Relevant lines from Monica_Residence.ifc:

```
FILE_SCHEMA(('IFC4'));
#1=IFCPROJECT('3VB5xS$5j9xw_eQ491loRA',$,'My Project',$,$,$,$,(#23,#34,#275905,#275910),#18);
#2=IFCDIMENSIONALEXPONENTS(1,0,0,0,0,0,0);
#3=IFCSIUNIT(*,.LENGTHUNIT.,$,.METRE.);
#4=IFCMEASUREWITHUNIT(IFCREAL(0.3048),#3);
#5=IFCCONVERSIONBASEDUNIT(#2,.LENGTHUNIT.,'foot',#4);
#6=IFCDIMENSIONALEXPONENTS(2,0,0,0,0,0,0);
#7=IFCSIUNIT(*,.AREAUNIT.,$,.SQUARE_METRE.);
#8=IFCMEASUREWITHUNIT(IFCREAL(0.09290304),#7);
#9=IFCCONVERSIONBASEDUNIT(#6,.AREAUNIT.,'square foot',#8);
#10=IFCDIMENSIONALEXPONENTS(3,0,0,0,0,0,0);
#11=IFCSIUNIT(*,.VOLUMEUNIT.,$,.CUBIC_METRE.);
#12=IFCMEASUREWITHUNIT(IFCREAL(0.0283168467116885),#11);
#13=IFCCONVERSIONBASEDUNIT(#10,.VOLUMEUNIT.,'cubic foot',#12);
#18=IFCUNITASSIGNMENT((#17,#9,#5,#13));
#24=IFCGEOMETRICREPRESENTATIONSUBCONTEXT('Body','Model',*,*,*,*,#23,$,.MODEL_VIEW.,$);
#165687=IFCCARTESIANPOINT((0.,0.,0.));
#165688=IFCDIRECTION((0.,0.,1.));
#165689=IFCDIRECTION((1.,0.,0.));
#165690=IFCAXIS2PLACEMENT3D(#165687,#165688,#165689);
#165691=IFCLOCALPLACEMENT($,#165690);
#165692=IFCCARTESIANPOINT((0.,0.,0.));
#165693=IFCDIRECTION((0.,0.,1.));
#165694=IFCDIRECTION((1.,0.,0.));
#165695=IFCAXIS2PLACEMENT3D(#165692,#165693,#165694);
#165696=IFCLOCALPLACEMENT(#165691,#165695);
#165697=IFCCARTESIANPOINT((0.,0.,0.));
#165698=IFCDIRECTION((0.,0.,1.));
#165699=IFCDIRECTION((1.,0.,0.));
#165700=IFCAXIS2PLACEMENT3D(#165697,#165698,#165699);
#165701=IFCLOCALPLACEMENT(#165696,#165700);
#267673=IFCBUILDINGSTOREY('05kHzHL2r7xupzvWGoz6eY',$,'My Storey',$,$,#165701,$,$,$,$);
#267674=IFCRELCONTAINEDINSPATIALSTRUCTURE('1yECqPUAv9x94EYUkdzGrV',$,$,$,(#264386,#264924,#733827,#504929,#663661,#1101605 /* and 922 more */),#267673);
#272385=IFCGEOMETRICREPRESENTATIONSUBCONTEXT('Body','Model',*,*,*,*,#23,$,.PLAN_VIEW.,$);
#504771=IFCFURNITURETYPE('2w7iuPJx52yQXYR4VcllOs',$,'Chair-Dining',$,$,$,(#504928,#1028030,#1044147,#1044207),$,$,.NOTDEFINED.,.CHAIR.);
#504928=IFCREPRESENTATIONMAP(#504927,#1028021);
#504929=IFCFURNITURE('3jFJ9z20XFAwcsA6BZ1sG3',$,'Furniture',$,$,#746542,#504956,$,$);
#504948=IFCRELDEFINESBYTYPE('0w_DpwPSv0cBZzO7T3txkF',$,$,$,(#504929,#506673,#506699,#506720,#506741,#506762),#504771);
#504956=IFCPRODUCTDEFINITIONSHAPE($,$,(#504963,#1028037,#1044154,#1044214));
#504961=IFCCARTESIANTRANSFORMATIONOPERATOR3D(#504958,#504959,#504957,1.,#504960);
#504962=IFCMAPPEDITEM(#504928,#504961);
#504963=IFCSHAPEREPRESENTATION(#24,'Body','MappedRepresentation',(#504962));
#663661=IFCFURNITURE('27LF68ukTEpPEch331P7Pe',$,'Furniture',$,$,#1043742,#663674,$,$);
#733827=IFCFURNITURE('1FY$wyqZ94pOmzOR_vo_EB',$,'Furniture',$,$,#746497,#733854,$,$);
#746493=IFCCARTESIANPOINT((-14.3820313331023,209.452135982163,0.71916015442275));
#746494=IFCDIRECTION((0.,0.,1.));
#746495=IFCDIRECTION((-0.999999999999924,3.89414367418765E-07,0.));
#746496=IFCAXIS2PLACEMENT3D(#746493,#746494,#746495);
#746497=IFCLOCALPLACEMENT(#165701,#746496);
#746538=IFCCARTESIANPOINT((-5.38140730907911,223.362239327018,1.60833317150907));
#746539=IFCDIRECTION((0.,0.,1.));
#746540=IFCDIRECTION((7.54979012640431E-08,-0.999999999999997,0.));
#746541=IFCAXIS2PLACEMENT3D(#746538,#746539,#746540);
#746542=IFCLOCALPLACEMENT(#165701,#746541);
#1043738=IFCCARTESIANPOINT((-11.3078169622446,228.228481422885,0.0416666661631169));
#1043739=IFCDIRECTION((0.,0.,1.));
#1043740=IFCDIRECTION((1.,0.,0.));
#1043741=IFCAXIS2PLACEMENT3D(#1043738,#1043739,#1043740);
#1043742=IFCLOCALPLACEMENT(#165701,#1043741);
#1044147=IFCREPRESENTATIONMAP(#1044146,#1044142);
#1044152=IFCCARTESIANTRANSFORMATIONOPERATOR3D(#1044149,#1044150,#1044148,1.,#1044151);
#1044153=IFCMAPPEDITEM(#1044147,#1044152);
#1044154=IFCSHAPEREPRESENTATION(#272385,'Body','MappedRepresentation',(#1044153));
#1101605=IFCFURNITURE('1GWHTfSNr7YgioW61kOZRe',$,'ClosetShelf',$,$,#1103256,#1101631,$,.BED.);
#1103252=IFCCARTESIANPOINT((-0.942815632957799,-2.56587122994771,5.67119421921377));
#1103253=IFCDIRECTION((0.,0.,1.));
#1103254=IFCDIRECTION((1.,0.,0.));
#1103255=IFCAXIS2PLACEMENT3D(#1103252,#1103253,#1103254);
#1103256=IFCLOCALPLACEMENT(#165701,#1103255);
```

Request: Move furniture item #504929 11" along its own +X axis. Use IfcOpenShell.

```python
import ifcopenshell
import ifcopenshell.api.geometry
import ifcopenshell.util.placement
import ifcopenshell.util.unit

model = ifcopenshell.open("Monica_Residence.ifc")
unit_scale = ifcopenshell.util.unit.calculate_unit_scale(model)

item = model.by_id(504929)
matrix = ifcopenshell.util.placement.get_local_placement(item.ObjectPlacement)
matrix[:3, 3] += matrix[:3, 0] * 11 * 0.0254 / unit_scale
ifcopenshell.api.geometry.edit_object_placement(model, product=item, matrix=matrix, is_si=False)

print(ifcopenshell.util.placement.get_local_placement(item.ObjectPlacement).round(3) + 0.0)

model.write("Monica_Residence_edited.ifc")
```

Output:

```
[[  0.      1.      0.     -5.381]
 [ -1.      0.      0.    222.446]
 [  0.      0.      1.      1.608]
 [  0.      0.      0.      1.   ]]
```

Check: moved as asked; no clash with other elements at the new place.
